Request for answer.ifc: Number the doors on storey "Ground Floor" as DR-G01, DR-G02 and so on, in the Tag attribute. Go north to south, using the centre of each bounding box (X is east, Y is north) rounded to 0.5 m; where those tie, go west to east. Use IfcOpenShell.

First a look at what the model holds.

```python
import ifcopenshell
import ifcopenshell.util.element
import ifcopenshell.util.placement

model = ifcopenshell.open("answer.ifc")
print(model.schema)
storey = next(s for s in model.by_type("IfcBuildingStorey") if s.Name == "Ground Floor")
doors = [e for e in ifcopenshell.util.element.get_decomposition(storey) if e.is_a("IfcDoor")]
for e in sorted(doors, key=lambda e: e.id()):
    origin = ifcopenshell.util.placement.get_local_placement(e.ObjectPlacement)[:3, 3]
    print(e.id(), e.Tag, e.Name, origin.round(2) + 0.0, sep=" | ")
```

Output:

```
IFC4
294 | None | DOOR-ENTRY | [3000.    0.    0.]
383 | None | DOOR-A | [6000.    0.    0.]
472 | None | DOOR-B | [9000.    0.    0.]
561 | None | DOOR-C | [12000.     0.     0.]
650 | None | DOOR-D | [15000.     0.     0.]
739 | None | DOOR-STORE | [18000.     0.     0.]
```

```python
import ifcopenshell
import ifcopenshell.geom
import ifcopenshell.util.element
import ifcopenshell.util.shape

model = ifcopenshell.open("answer.ifc")
settings = ifcopenshell.geom.settings()
settings.set("use-world-coords", True)


def centre(element):
    shape = ifcopenshell.geom.create_shape(settings, element)
    return ifcopenshell.util.shape.get_bbox_centroid(shape.geometry)


storey = next(s for s in model.by_type("IfcBuildingStorey") if s.Name == "Ground Floor")
doors = [e for e in ifcopenshell.util.element.get_decomposition(storey) if e.is_a("IfcDoor")]

# Insertion points can sit at a corner or the storey origin, so sort by the geometry (in metres).
centres = {e: centre(e) for e in doors}
doors.sort(key=lambda e: (-round(centres[e][1] / 0.5), centres[e][0]))

for i, e in enumerate(doors, start=1):
    number = f"DR-G{i:02d}"
    e.Tag = number
    print(e.id(), number)

model.write("answer_v2.ifc")
```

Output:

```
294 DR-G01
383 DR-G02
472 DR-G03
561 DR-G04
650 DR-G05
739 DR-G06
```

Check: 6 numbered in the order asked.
